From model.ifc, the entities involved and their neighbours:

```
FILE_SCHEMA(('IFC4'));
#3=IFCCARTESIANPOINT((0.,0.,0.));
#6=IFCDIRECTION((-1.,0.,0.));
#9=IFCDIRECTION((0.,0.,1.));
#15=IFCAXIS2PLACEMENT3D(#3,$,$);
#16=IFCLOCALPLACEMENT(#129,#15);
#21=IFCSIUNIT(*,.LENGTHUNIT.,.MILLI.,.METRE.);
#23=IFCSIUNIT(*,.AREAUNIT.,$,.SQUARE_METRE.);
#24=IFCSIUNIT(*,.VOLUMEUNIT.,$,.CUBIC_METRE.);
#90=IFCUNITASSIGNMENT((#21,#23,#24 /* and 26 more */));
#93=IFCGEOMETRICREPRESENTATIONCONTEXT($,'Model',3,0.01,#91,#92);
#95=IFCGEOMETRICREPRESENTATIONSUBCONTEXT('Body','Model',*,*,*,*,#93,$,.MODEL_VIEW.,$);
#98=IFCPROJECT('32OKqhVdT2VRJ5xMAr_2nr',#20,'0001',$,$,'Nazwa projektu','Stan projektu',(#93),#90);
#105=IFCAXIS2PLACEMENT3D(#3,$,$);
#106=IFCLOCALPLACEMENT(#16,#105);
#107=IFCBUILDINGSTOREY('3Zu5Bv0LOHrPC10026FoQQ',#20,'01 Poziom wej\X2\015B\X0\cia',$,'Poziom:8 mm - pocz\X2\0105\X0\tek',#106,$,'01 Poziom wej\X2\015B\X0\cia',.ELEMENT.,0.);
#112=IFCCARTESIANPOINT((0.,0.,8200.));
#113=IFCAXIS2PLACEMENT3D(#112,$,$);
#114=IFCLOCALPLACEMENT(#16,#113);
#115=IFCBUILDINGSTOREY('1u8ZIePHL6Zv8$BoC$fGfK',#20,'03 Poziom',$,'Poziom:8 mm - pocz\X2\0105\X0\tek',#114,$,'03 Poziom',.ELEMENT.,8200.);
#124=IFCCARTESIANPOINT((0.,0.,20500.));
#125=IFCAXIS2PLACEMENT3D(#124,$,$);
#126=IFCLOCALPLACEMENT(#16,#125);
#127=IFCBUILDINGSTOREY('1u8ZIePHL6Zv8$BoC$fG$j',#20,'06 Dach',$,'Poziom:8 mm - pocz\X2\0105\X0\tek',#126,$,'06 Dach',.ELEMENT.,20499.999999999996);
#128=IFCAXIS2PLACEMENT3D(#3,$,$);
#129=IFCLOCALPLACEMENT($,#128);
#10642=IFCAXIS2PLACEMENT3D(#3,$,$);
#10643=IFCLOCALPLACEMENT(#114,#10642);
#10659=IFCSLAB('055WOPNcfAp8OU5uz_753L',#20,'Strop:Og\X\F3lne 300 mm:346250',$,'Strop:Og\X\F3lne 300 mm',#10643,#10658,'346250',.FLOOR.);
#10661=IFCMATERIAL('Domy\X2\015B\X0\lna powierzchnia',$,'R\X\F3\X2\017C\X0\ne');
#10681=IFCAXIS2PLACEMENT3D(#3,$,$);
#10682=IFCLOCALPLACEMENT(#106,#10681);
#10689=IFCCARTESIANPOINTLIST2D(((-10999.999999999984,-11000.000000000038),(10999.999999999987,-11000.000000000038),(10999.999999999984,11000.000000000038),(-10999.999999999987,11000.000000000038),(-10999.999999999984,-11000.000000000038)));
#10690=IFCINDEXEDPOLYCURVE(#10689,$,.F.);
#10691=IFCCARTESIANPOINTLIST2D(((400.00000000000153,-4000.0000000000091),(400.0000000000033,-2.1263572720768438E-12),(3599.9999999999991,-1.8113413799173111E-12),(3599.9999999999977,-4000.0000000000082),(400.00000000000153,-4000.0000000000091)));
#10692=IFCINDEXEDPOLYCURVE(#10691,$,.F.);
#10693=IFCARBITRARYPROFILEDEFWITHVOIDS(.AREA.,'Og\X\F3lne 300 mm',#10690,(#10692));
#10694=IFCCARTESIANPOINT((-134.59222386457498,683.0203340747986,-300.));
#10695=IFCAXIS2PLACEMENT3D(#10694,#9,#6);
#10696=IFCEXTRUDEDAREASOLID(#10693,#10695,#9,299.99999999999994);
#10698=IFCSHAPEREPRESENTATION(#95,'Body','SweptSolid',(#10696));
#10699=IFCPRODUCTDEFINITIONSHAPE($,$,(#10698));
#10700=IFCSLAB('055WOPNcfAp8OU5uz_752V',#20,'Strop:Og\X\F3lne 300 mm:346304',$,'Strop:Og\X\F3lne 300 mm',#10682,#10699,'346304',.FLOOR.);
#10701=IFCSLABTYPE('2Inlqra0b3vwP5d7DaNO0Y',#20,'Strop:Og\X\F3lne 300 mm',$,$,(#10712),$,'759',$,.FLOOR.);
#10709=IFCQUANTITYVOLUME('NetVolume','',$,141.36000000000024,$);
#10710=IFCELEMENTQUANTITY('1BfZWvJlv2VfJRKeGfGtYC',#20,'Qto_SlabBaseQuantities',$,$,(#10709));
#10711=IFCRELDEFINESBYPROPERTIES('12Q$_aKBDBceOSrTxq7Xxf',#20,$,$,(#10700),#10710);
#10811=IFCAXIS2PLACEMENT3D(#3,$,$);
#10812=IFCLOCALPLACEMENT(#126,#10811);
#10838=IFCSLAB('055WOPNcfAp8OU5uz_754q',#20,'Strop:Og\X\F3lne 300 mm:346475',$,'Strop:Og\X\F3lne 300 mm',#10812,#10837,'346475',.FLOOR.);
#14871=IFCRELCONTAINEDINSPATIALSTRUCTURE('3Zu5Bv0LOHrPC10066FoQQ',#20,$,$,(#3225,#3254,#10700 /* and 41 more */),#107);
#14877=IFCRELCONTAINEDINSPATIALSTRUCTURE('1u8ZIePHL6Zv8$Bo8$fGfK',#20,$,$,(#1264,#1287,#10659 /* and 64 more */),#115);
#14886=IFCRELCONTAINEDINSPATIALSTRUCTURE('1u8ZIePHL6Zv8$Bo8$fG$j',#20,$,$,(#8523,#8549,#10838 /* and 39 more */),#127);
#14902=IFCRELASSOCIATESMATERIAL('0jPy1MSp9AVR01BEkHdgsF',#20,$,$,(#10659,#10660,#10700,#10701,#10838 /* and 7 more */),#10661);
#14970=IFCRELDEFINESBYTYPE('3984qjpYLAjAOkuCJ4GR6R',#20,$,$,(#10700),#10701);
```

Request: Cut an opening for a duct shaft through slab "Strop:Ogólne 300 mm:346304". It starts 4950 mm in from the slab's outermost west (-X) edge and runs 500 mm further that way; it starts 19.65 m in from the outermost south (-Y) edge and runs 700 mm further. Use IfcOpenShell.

```python
import numpy as np
import ifcopenshell
import ifcopenshell.api.feature
import ifcopenshell.api.geometry
import ifcopenshell.api.pset
import ifcopenshell.api.root
import ifcopenshell.geom
import ifcopenshell.util.element
import ifcopenshell.util.placement
import ifcopenshell.util.representation
import ifcopenshell.util.shape
import ifcopenshell.util.unit

model = ifcopenshell.open("model.ifc")
unit_scale = ifcopenshell.util.unit.calculate_unit_scale(model)
volume_scale = ifcopenshell.util.unit.calculate_unit_scale(model, "VOLUMEUNIT")
settings = ifcopenshell.geom.settings()


def volume(element):
    """Net volume in cubic metres, openings subtracted."""
    shape = ifcopenshell.geom.create_shape(settings, element)
    return ifcopenshell.util.shape.get_volume(shape.geometry)


slab = model.by_id(10700)
before = volume(slab)

# Extent in the slab's own axes, in metres. The edges named are its -X and -Y sides.
slab_shape = ifcopenshell.geom.create_shape(settings, slab)
vertices = ifcopenshell.util.shape.get_vertices(slab_shape.geometry)
x_min, y_min, bottom = vertices.min(axis=0)
top = vertices[:, 2].max()

opening = ifcopenshell.api.root.create_entity(model, ifc_class="IfcOpeningElement", name="Duct shaft opening", predefined_type="OPENING")
context = ifcopenshell.util.representation.get_context(model, "Model", "Body", "MODEL_VIEW")
width, depth = 0.5, 0.7
outline = [(0.0, 0.0), (width, 0.0), (width, depth), (0.0, depth), (0.0, 0.0)]
# Overshoot both faces by 50 mm so the cut is clean.
shape = ifcopenshell.api.geometry.add_slab_representation(
    model, context=context, depth=top - bottom + 0.1, polyline=outline
)
ifcopenshell.api.geometry.assign_representation(model, product=opening, representation=shape)

matrix = ifcopenshell.util.placement.get_local_placement(slab.ObjectPlacement)
matrix[:, 3] = matrix @ np.append(np.array([x_min + 4.95, y_min + 19.65, bottom - 0.05]) / unit_scale, 1.0)
ifcopenshell.api.geometry.edit_object_placement(model, product=opening, matrix=matrix, is_si=False)
ifcopenshell.api.feature.add_feature(model, feature=opening, element=slab)

after = volume(slab)

# Update the slab's stored quantities.
qto = model.by_id(ifcopenshell.util.element.get_pset(slab, "Qto_SlabBaseQuantities", should_inherit=False)["id"])
ifcopenshell.api.pset.edit_qto(model, qto=qto, properties={"NetVolume": after / volume_scale})

print(f"slab volume {before:.3f} -> {after:.3f} m3")

model.write("model_v2.ifc")
```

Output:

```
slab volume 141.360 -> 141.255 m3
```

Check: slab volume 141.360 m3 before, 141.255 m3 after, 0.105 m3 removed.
